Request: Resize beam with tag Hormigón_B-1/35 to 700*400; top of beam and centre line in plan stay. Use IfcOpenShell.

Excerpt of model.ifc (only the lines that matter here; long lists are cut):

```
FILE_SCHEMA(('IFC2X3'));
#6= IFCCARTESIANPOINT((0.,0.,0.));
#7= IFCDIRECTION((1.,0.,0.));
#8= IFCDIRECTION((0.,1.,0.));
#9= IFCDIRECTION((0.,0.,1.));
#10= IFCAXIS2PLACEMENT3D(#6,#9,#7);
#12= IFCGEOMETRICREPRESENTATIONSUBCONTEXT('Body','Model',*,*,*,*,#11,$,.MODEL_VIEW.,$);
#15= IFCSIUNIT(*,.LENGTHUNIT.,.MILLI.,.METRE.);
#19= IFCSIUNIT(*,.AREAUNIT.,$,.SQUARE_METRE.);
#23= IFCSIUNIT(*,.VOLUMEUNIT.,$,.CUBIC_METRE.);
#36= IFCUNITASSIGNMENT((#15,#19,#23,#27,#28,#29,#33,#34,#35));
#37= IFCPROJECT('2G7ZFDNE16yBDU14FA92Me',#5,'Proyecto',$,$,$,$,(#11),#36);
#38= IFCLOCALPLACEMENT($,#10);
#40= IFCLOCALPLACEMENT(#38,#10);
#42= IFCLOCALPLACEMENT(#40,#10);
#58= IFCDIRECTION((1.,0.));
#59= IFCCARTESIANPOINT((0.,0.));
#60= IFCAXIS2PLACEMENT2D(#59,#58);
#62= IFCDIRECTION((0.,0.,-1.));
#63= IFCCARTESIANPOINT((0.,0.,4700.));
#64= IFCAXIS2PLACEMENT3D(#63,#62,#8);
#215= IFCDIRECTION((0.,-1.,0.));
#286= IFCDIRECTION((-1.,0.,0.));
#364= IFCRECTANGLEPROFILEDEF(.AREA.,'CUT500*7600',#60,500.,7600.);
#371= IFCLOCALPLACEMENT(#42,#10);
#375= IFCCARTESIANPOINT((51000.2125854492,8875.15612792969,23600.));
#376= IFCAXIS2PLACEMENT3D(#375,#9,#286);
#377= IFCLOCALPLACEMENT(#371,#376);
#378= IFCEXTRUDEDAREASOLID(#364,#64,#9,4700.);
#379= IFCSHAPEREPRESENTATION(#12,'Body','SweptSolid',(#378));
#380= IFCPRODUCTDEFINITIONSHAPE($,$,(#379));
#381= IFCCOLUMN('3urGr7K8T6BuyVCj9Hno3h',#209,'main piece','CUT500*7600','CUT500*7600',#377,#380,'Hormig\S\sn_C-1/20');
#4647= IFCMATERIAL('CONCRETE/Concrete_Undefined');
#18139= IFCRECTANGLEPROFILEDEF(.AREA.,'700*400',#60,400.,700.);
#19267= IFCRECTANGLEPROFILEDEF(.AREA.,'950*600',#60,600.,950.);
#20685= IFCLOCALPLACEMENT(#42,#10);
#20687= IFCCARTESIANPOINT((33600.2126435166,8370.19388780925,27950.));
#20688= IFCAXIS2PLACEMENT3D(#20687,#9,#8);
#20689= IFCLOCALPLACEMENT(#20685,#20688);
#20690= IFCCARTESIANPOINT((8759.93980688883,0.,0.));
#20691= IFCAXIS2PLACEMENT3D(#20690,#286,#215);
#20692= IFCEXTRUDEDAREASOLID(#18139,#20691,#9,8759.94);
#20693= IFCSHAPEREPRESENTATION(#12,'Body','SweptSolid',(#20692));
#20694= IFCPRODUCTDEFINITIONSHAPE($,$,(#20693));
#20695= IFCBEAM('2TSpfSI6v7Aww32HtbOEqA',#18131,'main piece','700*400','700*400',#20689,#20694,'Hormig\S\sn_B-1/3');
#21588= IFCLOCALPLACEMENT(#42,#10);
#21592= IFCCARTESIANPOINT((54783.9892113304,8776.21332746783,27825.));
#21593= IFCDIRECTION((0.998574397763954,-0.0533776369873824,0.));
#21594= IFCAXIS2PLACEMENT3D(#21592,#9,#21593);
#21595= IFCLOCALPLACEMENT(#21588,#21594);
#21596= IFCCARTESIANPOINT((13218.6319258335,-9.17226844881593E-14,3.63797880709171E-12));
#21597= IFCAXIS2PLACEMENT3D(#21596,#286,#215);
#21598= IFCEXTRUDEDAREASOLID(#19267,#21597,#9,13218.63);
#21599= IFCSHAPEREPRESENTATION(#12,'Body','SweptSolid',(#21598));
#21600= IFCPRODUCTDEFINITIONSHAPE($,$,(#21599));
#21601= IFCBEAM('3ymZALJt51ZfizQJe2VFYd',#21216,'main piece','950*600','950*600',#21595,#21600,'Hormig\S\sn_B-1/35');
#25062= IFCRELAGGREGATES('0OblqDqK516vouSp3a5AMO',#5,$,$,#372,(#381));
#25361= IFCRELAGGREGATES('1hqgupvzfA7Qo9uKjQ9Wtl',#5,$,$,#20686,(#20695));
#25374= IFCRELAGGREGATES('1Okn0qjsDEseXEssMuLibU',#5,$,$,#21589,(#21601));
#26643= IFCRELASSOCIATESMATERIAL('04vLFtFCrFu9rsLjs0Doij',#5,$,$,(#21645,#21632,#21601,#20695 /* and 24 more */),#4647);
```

```python
import ifcopenshell
import ifcopenshell.util.element
import ifcopenshell.util.representation

model = ifcopenshell.open("model.ifc")

member = model.by_id(21601)
source = next(p for p in model.by_type("IfcRectangleProfileDef") if p.ProfileName == "700*400")

body = ifcopenshell.util.representation.get_representation(member, "Model", "Body")
solid = body.Items[0]
old_profile = solid.SweptArea

# Copy the section's sizes but keep this member's own profile position.
profile = ifcopenshell.util.element.copy(model, source)
# Profiles are centred, so shift by half the change in depth to hold the top.
shift = (old_profile.YDim - profile.YDim) / 2
x, y = old_profile.Position.Location.Coordinates
up = (0.0, 1.0)  # upwards, in the solid's own plane
location = model.createIfcCartesianPoint((x + up[0] * shift, y + up[1] * shift))
profile.Position = model.createIfcAxis2Placement2D(location, old_profile.Position.RefDirection)
solid.SweptArea = profile
if not model.get_total_inverses(old_profile):
    ifcopenshell.util.element.remove_deep2(model, old_profile)
member.Description = member.Description.replace("950*600", "700*400")
member.ObjectType = member.ObjectType.replace("950*600", "700*400")

print(solid.SweptArea)

model.write("model-out.ifc")
```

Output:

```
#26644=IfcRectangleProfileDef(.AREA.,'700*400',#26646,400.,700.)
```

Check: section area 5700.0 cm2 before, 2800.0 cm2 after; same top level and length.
